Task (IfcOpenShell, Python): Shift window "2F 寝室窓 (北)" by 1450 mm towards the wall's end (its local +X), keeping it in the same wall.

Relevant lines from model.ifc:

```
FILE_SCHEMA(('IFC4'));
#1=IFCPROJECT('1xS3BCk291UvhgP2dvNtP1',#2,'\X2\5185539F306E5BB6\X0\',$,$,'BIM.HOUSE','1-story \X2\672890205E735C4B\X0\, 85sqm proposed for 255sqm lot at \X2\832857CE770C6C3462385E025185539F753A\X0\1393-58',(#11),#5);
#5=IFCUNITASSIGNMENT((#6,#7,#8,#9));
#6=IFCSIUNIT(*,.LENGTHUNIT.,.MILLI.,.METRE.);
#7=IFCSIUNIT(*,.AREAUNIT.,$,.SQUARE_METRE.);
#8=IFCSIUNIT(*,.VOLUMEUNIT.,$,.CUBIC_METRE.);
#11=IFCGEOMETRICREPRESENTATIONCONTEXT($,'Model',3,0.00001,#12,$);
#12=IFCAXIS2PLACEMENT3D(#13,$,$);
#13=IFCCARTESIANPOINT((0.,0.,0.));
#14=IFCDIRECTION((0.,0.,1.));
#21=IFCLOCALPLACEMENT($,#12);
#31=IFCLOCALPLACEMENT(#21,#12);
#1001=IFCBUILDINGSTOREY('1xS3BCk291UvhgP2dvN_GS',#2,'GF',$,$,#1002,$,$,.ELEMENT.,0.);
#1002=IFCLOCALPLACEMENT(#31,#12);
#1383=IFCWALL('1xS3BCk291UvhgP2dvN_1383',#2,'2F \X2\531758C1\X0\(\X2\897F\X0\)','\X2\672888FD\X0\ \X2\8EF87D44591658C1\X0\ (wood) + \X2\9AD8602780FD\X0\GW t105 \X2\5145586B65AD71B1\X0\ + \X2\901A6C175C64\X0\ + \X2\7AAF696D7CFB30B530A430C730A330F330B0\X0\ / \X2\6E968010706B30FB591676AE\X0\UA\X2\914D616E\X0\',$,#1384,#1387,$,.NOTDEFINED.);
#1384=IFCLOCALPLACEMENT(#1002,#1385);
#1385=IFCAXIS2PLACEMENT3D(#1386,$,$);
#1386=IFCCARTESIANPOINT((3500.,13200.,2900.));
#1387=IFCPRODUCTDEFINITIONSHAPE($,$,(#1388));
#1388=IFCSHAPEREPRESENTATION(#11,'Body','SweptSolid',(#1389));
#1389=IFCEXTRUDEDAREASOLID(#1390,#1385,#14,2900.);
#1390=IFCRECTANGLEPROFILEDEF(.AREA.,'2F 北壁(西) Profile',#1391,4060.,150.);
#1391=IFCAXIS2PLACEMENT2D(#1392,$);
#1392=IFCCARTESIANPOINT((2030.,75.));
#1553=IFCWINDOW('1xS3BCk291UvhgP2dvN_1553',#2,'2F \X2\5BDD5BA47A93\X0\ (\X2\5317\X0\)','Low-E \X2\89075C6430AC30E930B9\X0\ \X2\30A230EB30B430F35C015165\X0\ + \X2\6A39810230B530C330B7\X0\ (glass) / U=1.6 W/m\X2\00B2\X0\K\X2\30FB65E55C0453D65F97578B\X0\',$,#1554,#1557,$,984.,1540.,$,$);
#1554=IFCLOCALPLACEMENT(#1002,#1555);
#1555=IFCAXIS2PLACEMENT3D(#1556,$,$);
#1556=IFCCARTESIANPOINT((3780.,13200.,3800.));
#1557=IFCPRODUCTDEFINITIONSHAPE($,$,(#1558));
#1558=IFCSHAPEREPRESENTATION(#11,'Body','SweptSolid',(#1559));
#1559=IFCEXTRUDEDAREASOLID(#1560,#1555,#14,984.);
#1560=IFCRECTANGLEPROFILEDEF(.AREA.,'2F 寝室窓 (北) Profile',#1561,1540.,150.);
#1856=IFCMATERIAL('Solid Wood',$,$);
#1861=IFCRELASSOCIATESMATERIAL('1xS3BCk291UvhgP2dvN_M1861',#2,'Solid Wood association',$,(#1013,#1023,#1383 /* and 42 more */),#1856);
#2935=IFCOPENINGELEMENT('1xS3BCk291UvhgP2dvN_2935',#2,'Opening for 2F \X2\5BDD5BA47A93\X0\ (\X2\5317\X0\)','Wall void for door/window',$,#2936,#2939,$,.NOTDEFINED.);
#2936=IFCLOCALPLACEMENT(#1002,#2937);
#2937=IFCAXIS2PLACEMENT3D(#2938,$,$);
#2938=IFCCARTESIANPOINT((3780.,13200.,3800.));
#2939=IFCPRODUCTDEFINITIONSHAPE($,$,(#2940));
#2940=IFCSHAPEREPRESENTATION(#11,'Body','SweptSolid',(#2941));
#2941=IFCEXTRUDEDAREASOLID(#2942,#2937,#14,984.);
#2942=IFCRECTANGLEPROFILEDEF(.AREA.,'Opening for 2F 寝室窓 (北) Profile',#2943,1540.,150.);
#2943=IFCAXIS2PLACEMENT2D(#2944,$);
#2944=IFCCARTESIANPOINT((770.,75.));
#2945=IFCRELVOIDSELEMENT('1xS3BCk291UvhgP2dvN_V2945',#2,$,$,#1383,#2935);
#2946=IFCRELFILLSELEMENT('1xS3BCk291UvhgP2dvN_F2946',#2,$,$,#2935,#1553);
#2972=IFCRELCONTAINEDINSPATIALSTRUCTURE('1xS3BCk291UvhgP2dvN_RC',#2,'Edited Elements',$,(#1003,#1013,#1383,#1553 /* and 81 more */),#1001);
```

```python
import ifcopenshell
import ifcopenshell.api.geometry
import ifcopenshell.util.placement
import ifcopenshell.util.unit

model = ifcopenshell.open("model.ifc")
unit_scale = ifcopenshell.util.unit.calculate_unit_scale(model)

window = model.by_id(1553)
opening = window.FillsVoids[0].RelatingOpeningElement
wall = opening.VoidsElements[0].RelatingBuildingElement

wall_matrix = ifcopenshell.util.placement.get_local_placement(wall.ObjectPlacement)
shift = wall_matrix[:3, 0] * 1.45 / unit_scale
before = ifcopenshell.util.placement.get_local_placement(window.ObjectPlacement)[:3, 3].copy()

# The window is not placed relative to its opening, so move both.
for product in (opening, window):
    matrix = ifcopenshell.util.placement.get_local_placement(product.ObjectPlacement)
    matrix[:3, 3] += shift
    ifcopenshell.api.geometry.edit_object_placement(model, product=product, matrix=matrix, is_si=False)

after = ifcopenshell.util.placement.get_local_placement(window.ObjectPlacement)[:3, 3]
print("window moved by", (after - before).round(3) + 0.0)

model.write("model-out.ifc")
```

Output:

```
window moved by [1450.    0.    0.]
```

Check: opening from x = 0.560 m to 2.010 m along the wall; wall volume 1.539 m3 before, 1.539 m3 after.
